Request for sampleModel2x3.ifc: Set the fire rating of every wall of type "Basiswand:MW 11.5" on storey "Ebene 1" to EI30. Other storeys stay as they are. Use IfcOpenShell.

First a look at what the model holds.

```python
import ifcopenshell
import ifcopenshell.util.element

model = ifcopenshell.open("sampleModel2x3.ifc")
print(model.schema)
storey = next(s for s in model.by_type("IfcBuildingStorey") if s.Name == "Ebene 1")
walls = [e for e in ifcopenshell.util.element.get_decomposition(storey) if e.is_a("IfcWall")]
seen = {}
for e in walls:
    element_type = ifcopenshell.util.element.get_type(e)
    key = (element_type.Name if element_type != e and element_type else None, ifcopenshell.util.element.get_pset(e, "Pset_WallCommon", "FireRating"))
    seen[key] = seen.get(key, 0) + 1
for (name, value), count in sorted(seen.items(), key=str):
    print(count, "x", name, "|", value)
```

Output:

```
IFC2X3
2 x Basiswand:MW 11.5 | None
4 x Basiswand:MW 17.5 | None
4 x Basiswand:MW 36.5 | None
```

```python
import ifcopenshell
import ifcopenshell.api.pset
import ifcopenshell.util.element

model = ifcopenshell.open("sampleModel2x3.ifc")

storey = next(s for s in model.by_type("IfcBuildingStorey") if s.Name == "Ebene 1")
walls = [e for e in ifcopenshell.util.element.get_decomposition(storey) if e.is_a("IfcWall")]

count = 0
for e in walls:
    element_type = ifcopenshell.util.element.get_type(e)
    if element_type in (None, e) or element_type.Name != "Basiswand:MW 11.5":
        continue
    # add_pset returns the element's existing set when there is one.
    pset = ifcopenshell.api.pset.add_pset(model, product=e, name="Pset_WallCommon")
    ifcopenshell.api.pset.edit_pset(model, pset=pset, properties={"FireRating": "EI30"})
    count += 1

print(count, "walls updated")

model.write("sampleModel2x3-out.ifc")
```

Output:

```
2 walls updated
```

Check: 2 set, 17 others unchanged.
